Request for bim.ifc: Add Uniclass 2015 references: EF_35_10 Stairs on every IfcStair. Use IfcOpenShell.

First a look at what the model holds.

```python
import ifcopenshell

model = ifcopenshell.open("bim.ifc")
print(model.schema)
print("classifications:", [c.Name for c in model.by_type("IfcClassification")])
for ifc_class in ("IfcDoor", "IfcRoof", "IfcStair", "IfcWall", "IfcWindow"):
    print(ifc_class, len(model.by_type(ifc_class)))
```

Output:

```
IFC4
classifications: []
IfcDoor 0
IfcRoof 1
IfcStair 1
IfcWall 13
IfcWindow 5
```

```python
import ifcopenshell
import ifcopenshell.api.classification

model = ifcopenshell.open("bim.ifc")

system = ifcopenshell.api.classification.add_classification(model, classification="Uniclass 2015")

codes = {
    "IfcStair": ("EF_35_10", "Stairs"),
}
for ifc_class, (code, name) in codes.items():
    products = model.by_type(ifc_class)
    ifcopenshell.api.classification.add_reference(
        model, products=products, classification=system, identification=code, name=name
    )
    print(code, len(products))

model.write("bim_rev.ifc")
```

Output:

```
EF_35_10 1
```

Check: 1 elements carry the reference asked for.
